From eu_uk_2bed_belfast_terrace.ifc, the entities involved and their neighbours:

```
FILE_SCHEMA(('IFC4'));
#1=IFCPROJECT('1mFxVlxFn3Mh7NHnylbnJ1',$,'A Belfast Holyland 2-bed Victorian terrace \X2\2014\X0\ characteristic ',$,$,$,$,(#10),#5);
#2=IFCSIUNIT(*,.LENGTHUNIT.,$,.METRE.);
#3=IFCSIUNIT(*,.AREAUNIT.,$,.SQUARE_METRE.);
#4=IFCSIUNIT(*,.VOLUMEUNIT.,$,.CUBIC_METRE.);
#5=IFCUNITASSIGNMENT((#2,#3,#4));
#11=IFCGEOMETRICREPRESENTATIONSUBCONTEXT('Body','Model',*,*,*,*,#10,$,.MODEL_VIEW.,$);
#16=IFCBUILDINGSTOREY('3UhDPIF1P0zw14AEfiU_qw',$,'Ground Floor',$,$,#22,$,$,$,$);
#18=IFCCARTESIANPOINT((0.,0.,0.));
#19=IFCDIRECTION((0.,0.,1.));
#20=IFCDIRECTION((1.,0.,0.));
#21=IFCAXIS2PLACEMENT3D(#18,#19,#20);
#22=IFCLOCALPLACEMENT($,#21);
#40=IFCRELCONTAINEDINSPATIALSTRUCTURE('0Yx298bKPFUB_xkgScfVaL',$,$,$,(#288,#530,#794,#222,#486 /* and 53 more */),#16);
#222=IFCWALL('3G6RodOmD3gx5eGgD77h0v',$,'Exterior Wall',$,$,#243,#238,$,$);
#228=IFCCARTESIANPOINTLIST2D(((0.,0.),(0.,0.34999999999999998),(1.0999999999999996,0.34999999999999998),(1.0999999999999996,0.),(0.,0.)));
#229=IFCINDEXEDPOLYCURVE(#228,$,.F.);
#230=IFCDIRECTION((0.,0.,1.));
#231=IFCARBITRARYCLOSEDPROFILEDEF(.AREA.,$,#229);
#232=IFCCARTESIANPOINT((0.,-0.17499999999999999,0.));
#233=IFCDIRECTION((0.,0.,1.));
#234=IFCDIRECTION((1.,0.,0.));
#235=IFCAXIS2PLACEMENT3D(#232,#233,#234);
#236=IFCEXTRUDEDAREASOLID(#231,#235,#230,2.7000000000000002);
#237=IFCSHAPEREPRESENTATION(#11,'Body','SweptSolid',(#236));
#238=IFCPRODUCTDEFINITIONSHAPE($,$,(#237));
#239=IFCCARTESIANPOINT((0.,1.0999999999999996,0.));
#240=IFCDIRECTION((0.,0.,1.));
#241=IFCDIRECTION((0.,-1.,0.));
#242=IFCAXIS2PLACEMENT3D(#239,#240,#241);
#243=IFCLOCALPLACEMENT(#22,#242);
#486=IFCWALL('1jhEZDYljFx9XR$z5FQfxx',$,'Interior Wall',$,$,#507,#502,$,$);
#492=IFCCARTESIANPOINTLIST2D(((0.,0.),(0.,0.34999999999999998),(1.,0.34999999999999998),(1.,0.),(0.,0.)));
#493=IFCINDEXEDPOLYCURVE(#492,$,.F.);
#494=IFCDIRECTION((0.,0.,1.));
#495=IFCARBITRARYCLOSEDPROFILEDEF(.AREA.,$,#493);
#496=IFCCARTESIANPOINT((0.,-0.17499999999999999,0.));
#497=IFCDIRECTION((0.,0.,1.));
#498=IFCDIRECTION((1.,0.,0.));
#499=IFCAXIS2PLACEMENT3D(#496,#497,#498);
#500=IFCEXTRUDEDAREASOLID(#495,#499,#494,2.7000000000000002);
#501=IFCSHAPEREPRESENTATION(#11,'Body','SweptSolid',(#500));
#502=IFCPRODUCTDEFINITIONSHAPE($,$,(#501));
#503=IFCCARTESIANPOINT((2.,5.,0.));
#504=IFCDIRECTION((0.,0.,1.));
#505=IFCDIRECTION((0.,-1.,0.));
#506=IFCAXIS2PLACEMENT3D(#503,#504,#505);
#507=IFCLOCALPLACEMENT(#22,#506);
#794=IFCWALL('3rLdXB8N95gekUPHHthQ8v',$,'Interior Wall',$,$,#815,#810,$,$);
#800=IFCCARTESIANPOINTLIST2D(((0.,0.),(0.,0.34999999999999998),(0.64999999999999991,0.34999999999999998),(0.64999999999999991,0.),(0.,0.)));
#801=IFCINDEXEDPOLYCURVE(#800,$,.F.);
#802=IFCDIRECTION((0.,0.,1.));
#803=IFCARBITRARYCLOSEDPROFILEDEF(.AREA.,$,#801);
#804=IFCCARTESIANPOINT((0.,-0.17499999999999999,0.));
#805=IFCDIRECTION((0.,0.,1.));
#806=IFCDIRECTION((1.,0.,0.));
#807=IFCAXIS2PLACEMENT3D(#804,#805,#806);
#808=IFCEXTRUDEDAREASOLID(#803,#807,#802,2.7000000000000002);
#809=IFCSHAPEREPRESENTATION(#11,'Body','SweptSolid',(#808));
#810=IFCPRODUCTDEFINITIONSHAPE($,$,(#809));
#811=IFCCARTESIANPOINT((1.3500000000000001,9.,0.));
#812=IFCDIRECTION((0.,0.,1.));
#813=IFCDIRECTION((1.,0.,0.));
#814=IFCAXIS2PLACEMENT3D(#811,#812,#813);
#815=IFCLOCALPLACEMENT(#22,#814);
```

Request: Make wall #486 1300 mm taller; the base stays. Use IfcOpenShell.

```python
import ifcopenshell
import ifcopenshell.geom
import ifcopenshell.util.representation
import ifcopenshell.util.shape

model = ifcopenshell.open("eu_uk_2bed_belfast_terrace.ifc")
settings = ifcopenshell.geom.settings()


def volume(element):
    """Net volume in cubic metres, openings subtracted."""
    shape = ifcopenshell.geom.create_shape(settings, element)
    return ifcopenshell.util.shape.get_volume(shape.geometry)


wall = model.by_guid("1jhEZDYljFx9XR$z5FQfxx")
before = volume(wall)

body = ifcopenshell.util.representation.get_representation(wall, "Model", "Body")
solid = body.Items[0]
old_height = solid.Depth
solid.Depth += 1.3
after = volume(wall)

print(f"height {old_height:g} -> {solid.Depth:g}, volume {before:.3f} -> {after:.3f} m3")

model.write("eu_uk_2bed_belfast_terrace_rev.ifc")
```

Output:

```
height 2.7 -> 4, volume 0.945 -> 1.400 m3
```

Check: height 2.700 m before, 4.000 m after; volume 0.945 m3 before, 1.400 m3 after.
